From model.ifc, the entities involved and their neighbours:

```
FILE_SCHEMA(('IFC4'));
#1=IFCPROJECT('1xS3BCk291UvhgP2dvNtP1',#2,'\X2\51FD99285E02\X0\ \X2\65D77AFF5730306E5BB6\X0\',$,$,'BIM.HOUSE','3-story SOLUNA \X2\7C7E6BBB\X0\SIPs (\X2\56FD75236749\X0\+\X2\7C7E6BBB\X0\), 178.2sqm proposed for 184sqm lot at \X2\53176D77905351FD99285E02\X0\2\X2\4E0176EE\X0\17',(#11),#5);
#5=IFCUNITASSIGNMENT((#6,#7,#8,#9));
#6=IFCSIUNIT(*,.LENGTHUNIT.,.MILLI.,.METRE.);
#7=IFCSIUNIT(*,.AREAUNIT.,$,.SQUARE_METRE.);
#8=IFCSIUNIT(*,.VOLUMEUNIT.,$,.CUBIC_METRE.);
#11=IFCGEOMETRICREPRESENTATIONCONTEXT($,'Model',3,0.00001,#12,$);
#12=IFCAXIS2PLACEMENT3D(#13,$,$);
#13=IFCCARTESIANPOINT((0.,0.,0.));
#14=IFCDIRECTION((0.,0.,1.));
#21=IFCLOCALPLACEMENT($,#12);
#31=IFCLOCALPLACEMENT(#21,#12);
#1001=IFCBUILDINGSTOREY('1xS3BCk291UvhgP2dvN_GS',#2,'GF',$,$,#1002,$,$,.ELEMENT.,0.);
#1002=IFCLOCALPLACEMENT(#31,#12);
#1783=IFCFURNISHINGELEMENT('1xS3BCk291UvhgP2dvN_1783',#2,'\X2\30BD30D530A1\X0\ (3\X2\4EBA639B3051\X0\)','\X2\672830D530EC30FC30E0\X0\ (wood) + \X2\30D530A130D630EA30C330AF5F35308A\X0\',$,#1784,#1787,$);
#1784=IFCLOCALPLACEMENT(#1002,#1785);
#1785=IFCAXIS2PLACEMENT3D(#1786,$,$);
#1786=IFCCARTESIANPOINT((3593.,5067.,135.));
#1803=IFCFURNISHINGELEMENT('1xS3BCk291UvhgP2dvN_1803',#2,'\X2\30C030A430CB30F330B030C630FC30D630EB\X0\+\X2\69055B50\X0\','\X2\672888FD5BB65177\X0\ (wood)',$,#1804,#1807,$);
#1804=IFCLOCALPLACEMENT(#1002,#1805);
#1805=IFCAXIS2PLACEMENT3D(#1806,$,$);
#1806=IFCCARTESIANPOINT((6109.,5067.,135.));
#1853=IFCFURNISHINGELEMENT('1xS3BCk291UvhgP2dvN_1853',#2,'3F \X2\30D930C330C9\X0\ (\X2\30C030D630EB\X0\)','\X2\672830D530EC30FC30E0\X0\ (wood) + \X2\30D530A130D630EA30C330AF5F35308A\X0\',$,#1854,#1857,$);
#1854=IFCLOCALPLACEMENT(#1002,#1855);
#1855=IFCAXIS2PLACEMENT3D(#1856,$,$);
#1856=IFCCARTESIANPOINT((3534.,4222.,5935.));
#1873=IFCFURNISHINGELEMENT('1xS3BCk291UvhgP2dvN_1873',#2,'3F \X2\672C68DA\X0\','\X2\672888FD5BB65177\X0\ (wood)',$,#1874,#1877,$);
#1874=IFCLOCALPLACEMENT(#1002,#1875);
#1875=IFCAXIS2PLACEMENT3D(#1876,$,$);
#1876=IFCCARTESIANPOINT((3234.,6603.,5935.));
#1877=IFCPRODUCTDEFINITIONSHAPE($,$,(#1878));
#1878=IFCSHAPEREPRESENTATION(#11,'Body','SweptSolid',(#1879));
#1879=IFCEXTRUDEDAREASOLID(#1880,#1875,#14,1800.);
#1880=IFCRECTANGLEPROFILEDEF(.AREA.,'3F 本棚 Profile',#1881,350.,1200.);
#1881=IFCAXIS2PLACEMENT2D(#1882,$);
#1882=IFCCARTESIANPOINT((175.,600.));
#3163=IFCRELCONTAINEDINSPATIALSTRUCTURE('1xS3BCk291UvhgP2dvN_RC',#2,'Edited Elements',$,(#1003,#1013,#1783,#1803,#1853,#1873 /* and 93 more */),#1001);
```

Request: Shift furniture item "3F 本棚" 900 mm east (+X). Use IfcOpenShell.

```python
import ifcopenshell
import ifcopenshell.api.geometry
import ifcopenshell.util.placement
import ifcopenshell.util.unit

model = ifcopenshell.open("model.ifc")
unit_scale = ifcopenshell.util.unit.calculate_unit_scale(model)

item = model.by_guid("1xS3BCk291UvhgP2dvN_1873")
matrix = ifcopenshell.util.placement.get_local_placement(item.ObjectPlacement)
matrix[0, 3] += 0.9 / unit_scale
ifcopenshell.api.geometry.edit_object_placement(model, product=item, matrix=matrix, is_si=False)

print(ifcopenshell.util.placement.get_local_placement(item.ObjectPlacement).round(3) + 0.0)

model.write("model_v2.ifc")
```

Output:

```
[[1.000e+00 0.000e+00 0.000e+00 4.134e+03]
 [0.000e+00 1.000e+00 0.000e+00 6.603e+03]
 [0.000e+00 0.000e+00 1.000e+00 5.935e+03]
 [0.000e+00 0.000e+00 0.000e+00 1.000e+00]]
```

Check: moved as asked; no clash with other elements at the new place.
